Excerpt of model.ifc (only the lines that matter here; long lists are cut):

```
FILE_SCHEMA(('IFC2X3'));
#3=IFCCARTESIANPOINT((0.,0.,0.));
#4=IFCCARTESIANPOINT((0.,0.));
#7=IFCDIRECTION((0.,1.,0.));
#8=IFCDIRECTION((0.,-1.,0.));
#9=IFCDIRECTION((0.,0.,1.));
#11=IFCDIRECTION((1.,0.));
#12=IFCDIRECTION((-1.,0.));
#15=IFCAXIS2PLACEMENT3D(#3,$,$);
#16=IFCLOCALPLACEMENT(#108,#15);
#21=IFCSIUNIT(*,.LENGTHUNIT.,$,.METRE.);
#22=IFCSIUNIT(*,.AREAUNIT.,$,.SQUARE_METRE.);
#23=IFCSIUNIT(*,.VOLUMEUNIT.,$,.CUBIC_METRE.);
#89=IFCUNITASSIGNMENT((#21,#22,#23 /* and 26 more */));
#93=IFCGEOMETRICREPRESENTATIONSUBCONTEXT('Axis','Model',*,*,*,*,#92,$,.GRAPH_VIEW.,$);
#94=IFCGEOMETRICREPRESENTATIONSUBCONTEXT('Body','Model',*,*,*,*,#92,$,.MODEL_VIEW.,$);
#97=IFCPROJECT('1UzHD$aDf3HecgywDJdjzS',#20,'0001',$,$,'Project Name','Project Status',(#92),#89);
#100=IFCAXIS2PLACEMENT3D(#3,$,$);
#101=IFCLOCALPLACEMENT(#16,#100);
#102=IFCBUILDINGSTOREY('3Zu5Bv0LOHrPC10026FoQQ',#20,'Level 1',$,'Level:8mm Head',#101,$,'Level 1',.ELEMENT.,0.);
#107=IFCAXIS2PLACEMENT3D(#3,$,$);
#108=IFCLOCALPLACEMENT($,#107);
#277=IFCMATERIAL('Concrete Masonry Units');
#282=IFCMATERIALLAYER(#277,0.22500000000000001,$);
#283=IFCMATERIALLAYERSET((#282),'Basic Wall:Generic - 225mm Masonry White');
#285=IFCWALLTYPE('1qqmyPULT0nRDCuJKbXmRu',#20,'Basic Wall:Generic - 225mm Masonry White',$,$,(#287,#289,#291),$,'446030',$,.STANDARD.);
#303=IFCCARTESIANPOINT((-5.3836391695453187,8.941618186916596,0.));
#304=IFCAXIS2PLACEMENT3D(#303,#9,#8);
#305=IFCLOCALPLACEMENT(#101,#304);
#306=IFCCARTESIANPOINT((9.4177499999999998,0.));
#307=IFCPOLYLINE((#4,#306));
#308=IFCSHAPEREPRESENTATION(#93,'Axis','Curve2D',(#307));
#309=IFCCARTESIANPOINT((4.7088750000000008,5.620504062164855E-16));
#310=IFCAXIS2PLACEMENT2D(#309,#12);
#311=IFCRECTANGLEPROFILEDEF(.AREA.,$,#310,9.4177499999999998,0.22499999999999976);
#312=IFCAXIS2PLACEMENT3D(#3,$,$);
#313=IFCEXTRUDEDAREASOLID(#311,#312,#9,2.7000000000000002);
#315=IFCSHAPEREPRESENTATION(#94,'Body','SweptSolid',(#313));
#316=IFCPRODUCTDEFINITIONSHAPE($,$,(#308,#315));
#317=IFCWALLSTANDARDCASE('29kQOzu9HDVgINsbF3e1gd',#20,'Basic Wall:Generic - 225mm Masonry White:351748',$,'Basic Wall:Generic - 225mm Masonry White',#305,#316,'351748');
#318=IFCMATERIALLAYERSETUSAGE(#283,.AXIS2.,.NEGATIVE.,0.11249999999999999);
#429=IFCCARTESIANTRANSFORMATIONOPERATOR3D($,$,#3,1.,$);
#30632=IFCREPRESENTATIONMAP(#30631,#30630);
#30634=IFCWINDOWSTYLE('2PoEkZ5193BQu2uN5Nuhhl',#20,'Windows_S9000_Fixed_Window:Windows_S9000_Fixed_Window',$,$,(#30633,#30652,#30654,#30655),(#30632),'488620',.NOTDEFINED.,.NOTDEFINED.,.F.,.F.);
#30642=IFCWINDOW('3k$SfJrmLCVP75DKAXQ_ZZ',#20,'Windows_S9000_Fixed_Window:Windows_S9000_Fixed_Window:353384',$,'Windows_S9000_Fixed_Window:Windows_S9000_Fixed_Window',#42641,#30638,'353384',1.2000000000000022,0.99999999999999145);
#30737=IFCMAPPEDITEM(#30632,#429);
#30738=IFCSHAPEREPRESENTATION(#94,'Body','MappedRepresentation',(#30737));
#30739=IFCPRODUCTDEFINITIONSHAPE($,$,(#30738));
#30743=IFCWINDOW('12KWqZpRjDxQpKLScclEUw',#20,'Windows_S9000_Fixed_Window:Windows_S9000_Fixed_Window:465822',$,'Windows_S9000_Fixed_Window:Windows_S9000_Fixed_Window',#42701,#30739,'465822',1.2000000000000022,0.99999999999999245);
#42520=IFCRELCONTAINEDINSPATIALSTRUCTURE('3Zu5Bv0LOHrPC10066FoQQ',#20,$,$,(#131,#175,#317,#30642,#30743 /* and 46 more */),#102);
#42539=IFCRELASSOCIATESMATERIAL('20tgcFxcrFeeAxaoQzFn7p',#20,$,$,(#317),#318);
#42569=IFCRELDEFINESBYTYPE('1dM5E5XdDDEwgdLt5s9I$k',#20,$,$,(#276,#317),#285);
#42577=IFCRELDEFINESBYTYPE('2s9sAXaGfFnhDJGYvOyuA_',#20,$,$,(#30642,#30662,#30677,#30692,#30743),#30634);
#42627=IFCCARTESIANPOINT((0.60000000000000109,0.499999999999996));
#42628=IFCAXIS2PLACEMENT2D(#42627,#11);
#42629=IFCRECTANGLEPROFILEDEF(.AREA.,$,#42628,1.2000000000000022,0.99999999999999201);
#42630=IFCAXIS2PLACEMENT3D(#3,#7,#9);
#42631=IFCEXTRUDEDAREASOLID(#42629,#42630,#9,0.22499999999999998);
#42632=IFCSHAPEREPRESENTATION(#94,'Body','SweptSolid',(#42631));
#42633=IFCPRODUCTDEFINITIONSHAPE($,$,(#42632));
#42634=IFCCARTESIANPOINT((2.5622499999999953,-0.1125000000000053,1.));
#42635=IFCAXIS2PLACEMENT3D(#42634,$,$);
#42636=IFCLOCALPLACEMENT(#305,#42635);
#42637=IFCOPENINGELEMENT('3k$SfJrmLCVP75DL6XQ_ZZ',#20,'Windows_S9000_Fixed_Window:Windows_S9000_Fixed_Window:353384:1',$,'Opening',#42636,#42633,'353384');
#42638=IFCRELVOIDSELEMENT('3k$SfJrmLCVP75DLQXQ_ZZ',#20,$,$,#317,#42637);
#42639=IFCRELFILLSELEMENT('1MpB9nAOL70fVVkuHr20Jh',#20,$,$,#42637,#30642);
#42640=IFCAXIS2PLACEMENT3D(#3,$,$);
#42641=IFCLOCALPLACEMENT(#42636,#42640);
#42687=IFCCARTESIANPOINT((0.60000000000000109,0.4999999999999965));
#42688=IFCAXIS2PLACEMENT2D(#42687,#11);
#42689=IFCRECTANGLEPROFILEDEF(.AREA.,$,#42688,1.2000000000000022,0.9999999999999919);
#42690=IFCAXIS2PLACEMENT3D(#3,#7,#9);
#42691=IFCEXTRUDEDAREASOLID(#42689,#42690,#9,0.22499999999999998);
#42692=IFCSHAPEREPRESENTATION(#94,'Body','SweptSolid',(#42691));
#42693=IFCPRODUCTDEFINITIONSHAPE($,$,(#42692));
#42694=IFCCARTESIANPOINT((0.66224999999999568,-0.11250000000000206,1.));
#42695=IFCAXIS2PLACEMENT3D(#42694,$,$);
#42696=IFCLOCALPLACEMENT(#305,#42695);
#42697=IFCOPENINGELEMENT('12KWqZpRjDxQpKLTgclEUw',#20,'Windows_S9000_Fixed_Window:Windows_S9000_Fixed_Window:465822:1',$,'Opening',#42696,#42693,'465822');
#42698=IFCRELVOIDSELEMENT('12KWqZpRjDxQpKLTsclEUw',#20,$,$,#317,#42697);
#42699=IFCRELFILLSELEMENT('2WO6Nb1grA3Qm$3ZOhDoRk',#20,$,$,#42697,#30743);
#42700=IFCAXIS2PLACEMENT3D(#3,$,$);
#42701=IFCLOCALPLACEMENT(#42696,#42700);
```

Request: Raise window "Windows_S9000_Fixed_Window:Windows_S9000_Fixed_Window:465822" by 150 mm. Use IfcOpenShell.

```python
import numpy as np
import ifcopenshell
import ifcopenshell.api.geometry
import ifcopenshell.util.placement
import ifcopenshell.util.unit

model = ifcopenshell.open("model.ifc")
unit_scale = ifcopenshell.util.unit.calculate_unit_scale(model)

window = model.by_id(30743)
opening = window.FillsVoids[0].RelatingOpeningElement
dz = 0.15

shift = np.array([0.0, 0.0, dz])
# The window is placed relative to its opening, so it follows when the opening moves.
matrix = ifcopenshell.util.placement.get_local_placement(opening.ObjectPlacement)
matrix[:3, 3] += shift
ifcopenshell.api.geometry.edit_object_placement(
    model, product=opening, matrix=matrix, is_si=False, should_transform_children=True
)

print(f"moved by {dz * unit_scale:+.3f} m")

model.write("model_edited.ifc")
```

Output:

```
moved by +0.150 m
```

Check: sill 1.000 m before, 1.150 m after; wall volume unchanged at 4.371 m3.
